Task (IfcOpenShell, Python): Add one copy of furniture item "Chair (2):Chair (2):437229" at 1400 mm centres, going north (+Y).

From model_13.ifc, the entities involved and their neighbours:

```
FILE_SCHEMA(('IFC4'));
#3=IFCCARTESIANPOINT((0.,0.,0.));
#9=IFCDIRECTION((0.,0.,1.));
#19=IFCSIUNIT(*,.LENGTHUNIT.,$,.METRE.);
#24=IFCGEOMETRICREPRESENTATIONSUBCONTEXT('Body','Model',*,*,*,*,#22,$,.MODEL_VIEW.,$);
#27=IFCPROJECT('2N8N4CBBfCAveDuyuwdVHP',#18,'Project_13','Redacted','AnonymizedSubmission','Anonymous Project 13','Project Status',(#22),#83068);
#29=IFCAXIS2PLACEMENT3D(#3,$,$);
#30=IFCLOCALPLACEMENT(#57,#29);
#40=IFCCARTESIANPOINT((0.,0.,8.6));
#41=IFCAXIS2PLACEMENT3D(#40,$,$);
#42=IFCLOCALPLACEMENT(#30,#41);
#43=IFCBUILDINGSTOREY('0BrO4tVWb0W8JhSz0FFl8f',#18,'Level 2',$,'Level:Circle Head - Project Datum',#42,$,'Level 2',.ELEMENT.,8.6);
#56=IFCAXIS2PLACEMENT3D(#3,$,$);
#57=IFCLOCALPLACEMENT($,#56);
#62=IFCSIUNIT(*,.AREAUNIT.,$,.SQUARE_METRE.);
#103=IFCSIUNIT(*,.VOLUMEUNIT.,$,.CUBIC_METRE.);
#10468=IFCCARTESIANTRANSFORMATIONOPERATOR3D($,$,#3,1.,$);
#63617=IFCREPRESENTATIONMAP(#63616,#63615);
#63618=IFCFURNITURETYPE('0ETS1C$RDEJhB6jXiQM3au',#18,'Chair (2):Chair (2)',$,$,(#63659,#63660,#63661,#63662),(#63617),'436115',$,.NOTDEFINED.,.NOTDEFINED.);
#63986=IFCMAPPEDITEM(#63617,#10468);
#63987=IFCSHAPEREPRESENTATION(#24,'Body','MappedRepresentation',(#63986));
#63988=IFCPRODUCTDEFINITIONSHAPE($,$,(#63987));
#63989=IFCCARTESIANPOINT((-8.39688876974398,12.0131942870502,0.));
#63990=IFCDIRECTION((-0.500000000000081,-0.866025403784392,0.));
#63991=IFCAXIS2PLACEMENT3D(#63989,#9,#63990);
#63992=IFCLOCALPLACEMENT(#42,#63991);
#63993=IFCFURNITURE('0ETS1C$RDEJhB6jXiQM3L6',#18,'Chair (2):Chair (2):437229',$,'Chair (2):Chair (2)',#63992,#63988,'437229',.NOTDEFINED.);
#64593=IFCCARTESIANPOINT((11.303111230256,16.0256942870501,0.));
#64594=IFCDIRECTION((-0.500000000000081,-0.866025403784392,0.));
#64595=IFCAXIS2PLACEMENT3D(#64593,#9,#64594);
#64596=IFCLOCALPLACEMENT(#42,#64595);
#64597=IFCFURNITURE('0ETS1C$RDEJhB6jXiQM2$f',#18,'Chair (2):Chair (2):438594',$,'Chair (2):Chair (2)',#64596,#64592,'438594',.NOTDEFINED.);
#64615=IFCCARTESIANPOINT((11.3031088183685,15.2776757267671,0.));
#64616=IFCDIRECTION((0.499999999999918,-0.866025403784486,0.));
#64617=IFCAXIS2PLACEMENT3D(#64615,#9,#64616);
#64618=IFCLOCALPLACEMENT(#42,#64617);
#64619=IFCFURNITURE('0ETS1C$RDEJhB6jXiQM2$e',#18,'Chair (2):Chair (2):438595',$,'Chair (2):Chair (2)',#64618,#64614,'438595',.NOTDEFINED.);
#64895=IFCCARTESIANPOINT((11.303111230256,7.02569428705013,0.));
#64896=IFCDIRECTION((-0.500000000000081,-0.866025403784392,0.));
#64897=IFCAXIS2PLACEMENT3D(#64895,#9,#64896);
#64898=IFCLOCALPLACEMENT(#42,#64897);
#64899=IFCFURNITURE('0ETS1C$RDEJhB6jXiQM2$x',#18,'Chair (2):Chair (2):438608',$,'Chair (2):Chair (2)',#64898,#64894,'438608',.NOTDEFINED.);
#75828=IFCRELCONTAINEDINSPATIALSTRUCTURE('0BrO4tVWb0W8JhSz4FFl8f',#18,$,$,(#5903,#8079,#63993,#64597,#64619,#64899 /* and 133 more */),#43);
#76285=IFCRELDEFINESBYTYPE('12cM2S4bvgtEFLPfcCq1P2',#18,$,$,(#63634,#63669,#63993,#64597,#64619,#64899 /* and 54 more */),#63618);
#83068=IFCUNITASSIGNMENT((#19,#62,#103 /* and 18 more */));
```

```python
import numpy as np
import ifcopenshell
import ifcopenshell.api.geometry
import ifcopenshell.api.root
import ifcopenshell.util.element
import ifcopenshell.util.placement
import ifcopenshell.util.unit

model = ifcopenshell.open("model_13.ifc")
unit_scale = ifcopenshell.util.unit.calculate_unit_scale(model)


def reuse_history(source, copy):
    """copy_class also copies each property set's owner history, people and application; keep the originals."""
    for rel in copy.IsDefinedBy:
        if rel.is_a("IfcRelDefinesByProperties") and (history := rel.RelatingPropertyDefinition.OwnerHistory):
            rel.RelatingPropertyDefinition.OwnerHistory = source.OwnerHistory
            ifcopenshell.util.element.remove_deep2(model, history)


source = model.by_guid("0ETS1C$RDEJhB6jXiQM3L6")
base = ifcopenshell.util.placement.get_local_placement(source.ObjectPlacement)
step = np.array([0.0, 1.0, 0.0]) * 1.4 / unit_scale

for i in range(1, 2):
    copy = ifcopenshell.api.root.copy_class(model, product=source)
    copy.Representation = ifcopenshell.util.element.copy_deep(
        model, source.Representation, exclude=["IfcGeometricRepresentationContext", "IfcRepresentationMap"]
    )
    copy.Name = "Chair (2):Chair (2)"
    copy.Tag = None
    reuse_history(source, copy)
    matrix = base.copy()
    matrix[:3, 3] += i * step
    print("added at", matrix[:3, 3].round(3) + 0.0)
    ifcopenshell.api.geometry.edit_object_placement(model, product=copy, matrix=matrix, is_si=False)

model.write("model_13_edited.ifc")
```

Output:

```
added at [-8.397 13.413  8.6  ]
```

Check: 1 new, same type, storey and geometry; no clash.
